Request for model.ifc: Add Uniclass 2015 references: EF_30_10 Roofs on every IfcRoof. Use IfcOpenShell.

First a look at what the model holds.

```python
import ifcopenshell

model = ifcopenshell.open("model.ifc")
print(model.schema)
print("classifications:", [c.Name for c in model.by_type("IfcClassification")])
for ifc_class in ("IfcDoor", "IfcRoof", "IfcStair", "IfcWall", "IfcWindow"):
    print(ifc_class, len(model.by_type(ifc_class)))
```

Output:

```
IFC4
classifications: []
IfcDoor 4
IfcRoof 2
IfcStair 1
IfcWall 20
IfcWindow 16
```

```python
import ifcopenshell
import ifcopenshell.api.classification

model = ifcopenshell.open("model.ifc")

system = ifcopenshell.api.classification.add_classification(model, classification="Uniclass 2015")

codes = {
    "IfcRoof": ("EF_30_10", "Roofs"),
}
for ifc_class, (code, name) in codes.items():
    products = model.by_type(ifc_class)
    ifcopenshell.api.classification.add_reference(
        model, products=products, classification=system, identification=code, name=name
    )
    print(code, len(products))

model.write("model_edited.ifc")
```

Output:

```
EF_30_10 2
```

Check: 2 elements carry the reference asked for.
